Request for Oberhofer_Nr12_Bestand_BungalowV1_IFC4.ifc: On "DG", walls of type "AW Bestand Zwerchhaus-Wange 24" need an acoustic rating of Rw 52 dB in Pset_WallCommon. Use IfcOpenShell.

First a look at what the model holds.

```python
import ifcopenshell
import ifcopenshell.util.element

model = ifcopenshell.open("Oberhofer_Nr12_Bestand_BungalowV1_IFC4.ifc")
print(model.schema)
storey = next(s for s in model.by_type("IfcBuildingStorey") if s.Name == "DG")
walls = [e for e in ifcopenshell.util.element.get_decomposition(storey) if e.is_a("IfcWall")]
seen = {}
for e in walls:
    element_type = ifcopenshell.util.element.get_type(e)
    key = (element_type.Name if element_type != e and element_type else None, ifcopenshell.util.element.get_pset(e, "Pset_WallCommon", "AcousticRating"))
    seen[key] = seen.get(key, 0) + 1
for (name, value), count in sorted(seen.items(), key=str):
    print(count, "x", name, "|", value)
```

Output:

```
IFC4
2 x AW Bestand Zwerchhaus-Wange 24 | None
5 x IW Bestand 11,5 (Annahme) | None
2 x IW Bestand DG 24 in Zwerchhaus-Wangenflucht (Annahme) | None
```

```python
import ifcopenshell
import ifcopenshell.api.pset
import ifcopenshell.util.element

model = ifcopenshell.open("Oberhofer_Nr12_Bestand_BungalowV1_IFC4.ifc")

storey = next(s for s in model.by_type("IfcBuildingStorey") if s.Name == "DG")
walls = [e for e in ifcopenshell.util.element.get_decomposition(storey) if e.is_a("IfcWall")]

count = 0
for e in walls:
    element_type = ifcopenshell.util.element.get_type(e)
    if element_type in (None, e) or element_type.Name != "AW Bestand Zwerchhaus-Wange 24":
        continue
    # add_pset returns the element's existing set when there is one.
    pset = ifcopenshell.api.pset.add_pset(model, product=e, name="Pset_WallCommon")
    ifcopenshell.api.pset.edit_pset(model, pset=pset, properties={"AcousticRating": "Rw 52 dB"})
    count += 1

print(count, "walls updated")

model.write("Oberhofer_Nr12_Bestand_BungalowV1_IFC4-out.ifc")
```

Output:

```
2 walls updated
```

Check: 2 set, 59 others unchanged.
